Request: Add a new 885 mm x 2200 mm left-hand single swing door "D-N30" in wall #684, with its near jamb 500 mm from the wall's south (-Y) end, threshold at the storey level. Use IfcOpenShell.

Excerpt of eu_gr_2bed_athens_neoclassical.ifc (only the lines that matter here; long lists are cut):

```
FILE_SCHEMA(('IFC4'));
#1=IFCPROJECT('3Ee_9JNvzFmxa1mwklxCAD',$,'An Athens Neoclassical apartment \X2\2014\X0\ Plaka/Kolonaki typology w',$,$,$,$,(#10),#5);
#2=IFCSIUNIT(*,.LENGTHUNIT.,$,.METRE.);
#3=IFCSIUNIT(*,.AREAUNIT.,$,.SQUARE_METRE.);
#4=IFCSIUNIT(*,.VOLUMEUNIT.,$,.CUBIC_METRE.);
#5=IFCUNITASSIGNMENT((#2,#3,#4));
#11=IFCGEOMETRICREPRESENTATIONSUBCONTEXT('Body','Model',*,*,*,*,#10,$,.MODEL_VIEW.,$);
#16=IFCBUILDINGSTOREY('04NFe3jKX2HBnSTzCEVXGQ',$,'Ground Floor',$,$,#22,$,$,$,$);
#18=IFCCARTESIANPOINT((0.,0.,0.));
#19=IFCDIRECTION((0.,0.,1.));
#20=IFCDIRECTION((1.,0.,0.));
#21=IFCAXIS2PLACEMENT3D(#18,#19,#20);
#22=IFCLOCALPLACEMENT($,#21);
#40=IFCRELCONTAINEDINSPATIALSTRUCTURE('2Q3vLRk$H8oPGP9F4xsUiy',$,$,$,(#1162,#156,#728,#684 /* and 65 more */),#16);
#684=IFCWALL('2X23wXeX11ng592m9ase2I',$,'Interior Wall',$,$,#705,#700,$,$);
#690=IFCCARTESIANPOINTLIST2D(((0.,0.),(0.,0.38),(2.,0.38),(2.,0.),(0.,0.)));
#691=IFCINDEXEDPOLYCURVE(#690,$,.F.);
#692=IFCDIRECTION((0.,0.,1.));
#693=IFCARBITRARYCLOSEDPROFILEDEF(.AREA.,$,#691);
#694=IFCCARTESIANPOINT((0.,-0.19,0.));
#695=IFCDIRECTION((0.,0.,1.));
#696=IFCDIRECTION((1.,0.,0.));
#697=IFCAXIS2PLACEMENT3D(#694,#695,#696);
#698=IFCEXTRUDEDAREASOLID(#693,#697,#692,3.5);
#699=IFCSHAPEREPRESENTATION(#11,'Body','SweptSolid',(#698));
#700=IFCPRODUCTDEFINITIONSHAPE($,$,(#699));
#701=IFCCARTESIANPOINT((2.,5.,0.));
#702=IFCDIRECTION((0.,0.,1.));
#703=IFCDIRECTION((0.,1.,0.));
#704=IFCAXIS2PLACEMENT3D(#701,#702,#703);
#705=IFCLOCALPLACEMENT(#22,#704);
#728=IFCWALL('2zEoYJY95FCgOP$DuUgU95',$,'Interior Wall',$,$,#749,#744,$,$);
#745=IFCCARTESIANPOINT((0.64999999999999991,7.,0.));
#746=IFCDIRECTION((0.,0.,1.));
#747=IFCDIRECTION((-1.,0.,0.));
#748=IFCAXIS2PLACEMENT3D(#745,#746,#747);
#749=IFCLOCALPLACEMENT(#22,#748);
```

```python
import numpy as np
import ifcopenshell
import ifcopenshell.api.feature
import ifcopenshell.api.geometry
import ifcopenshell.api.root
import ifcopenshell.api.spatial
import ifcopenshell.geom
import ifcopenshell.util.element
import ifcopenshell.util.placement
import ifcopenshell.util.representation
import ifcopenshell.util.shape
import ifcopenshell.util.unit

model = ifcopenshell.open("eu_gr_2bed_athens_neoclassical.ifc")
unit_scale = ifcopenshell.util.unit.calculate_unit_scale(model)
settings = ifcopenshell.geom.settings()


def volume(element):
    """Net volume in cubic metres, openings subtracted."""
    shape = ifcopenshell.geom.create_shape(settings, element)
    return ifcopenshell.util.shape.get_volume(shape.geometry)


wall = model.by_guid("2X23wXeX11ng592m9ase2I")
storey = ifcopenshell.util.element.get_container(wall, ifc_class="IfcBuildingStorey")
context = ifcopenshell.util.representation.get_context(model, "Model", "Body", "MODEL_VIEW")
before = volume(wall)

width, height, from_end, sill = 0.885, 2.2, 0.5, 0.0  # metres

# The wall runs along its own X axis, and the end named is its -X end.
wall_shape = ifcopenshell.geom.create_shape(settings, wall)
x, y, z = ifcopenshell.util.shape.get_vertices(wall_shape.geometry).T
start = x.min() + from_end
face, thickness = float(y.min()), float(y.max() - y.min())
wall_matrix = ifcopenshell.util.placement.get_local_placement(wall.ObjectPlacement)
level = ifcopenshell.util.placement.get_local_placement(storey.ObjectPlacement)[2, 3]


def in_wall(x, y):
    """Placement at x, y metres in the wall's axes, at sill height."""
    matrix = wall_matrix.copy()
    matrix[:, 3] = wall_matrix @ np.array([x / unit_scale, y / unit_scale, 0.0, 1.0])
    matrix[2, 3] = level + sill / unit_scale
    return matrix


# Opening: a box that overshoots both wall faces by 50 mm.
opening = ifcopenshell.api.root.create_entity(model, ifc_class="IfcOpeningElement", predefined_type="OPENING")
box = ifcopenshell.api.geometry.add_wall_representation(
    model, context=context, length=width, height=height, thickness=thickness + 0.1
)
ifcopenshell.api.geometry.assign_representation(model, product=opening, representation=box)
ifcopenshell.api.geometry.edit_object_placement(model, product=opening, matrix=in_wall(start, face - 0.05), is_si=False)
ifcopenshell.api.feature.add_feature(model, feature=opening, element=wall)

door = ifcopenshell.api.root.create_entity(model, ifc_class="IfcDoor", name="D-N30", predefined_type="DOOR")
door.OverallWidth, door.OverallHeight = width / unit_scale, height / unit_scale
door.OperationType = "SINGLE_SWING_LEFT"
body = ifcopenshell.api.geometry.add_door_representation(
    model,
    context=context,
    overall_width=door.OverallWidth,
    overall_height=door.OverallHeight,
    operation_type="SINGLE_SWING_LEFT",
    lining_properties={"LiningDepth": thickness / unit_scale, "ThresholdDepth": thickness / unit_scale},
)
ifcopenshell.api.geometry.assign_representation(model, product=door, representation=body)
ifcopenshell.api.spatial.assign_container(model, products=[door], relating_structure=storey)
ifcopenshell.api.feature.add_filling(model, opening=opening, element=door)

# The lining spans the wall, so the door starts at the wall face.
ifcopenshell.api.geometry.edit_object_placement(model, product=door, matrix=in_wall(start, face), is_si=False)

after = volume(wall)

print(f"wall volume {before:.3f} -> {after:.3f} m3")

model.write("eu_gr_2bed_athens_neoclassical-out.ifc")
```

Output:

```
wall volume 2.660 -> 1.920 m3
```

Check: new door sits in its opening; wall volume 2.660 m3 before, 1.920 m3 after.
